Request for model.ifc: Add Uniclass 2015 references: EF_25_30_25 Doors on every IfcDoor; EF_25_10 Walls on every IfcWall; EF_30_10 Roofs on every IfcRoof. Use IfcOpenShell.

First a look at what the model holds.

```python
import ifcopenshell

model = ifcopenshell.open("model.ifc")
print(model.schema)
print("classifications:", [c.Name for c in model.by_type("IfcClassification")])
for ifc_class in ("IfcDoor", "IfcRoof", "IfcStair", "IfcWall", "IfcWindow"):
    print(ifc_class, len(model.by_type(ifc_class)))
```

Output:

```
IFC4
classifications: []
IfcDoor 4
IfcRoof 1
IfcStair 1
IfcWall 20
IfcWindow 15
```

```python
import ifcopenshell
import ifcopenshell.api.classification

model = ifcopenshell.open("model.ifc")

system = ifcopenshell.api.classification.add_classification(model, classification="Uniclass 2015")

codes = {
    "IfcDoor": ("EF_25_30_25", "Doors"),
    "IfcWall": ("EF_25_10", "Walls"),
    "IfcRoof": ("EF_30_10", "Roofs"),
}
for ifc_class, (code, name) in codes.items():
    products = model.by_type(ifc_class)
    ifcopenshell.api.classification.add_reference(
        model, products=products, classification=system, identification=code, name=name
    )
    print(code, len(products))

model.write("model_updated.ifc")
```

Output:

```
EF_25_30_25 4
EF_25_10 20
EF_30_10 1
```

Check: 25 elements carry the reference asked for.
